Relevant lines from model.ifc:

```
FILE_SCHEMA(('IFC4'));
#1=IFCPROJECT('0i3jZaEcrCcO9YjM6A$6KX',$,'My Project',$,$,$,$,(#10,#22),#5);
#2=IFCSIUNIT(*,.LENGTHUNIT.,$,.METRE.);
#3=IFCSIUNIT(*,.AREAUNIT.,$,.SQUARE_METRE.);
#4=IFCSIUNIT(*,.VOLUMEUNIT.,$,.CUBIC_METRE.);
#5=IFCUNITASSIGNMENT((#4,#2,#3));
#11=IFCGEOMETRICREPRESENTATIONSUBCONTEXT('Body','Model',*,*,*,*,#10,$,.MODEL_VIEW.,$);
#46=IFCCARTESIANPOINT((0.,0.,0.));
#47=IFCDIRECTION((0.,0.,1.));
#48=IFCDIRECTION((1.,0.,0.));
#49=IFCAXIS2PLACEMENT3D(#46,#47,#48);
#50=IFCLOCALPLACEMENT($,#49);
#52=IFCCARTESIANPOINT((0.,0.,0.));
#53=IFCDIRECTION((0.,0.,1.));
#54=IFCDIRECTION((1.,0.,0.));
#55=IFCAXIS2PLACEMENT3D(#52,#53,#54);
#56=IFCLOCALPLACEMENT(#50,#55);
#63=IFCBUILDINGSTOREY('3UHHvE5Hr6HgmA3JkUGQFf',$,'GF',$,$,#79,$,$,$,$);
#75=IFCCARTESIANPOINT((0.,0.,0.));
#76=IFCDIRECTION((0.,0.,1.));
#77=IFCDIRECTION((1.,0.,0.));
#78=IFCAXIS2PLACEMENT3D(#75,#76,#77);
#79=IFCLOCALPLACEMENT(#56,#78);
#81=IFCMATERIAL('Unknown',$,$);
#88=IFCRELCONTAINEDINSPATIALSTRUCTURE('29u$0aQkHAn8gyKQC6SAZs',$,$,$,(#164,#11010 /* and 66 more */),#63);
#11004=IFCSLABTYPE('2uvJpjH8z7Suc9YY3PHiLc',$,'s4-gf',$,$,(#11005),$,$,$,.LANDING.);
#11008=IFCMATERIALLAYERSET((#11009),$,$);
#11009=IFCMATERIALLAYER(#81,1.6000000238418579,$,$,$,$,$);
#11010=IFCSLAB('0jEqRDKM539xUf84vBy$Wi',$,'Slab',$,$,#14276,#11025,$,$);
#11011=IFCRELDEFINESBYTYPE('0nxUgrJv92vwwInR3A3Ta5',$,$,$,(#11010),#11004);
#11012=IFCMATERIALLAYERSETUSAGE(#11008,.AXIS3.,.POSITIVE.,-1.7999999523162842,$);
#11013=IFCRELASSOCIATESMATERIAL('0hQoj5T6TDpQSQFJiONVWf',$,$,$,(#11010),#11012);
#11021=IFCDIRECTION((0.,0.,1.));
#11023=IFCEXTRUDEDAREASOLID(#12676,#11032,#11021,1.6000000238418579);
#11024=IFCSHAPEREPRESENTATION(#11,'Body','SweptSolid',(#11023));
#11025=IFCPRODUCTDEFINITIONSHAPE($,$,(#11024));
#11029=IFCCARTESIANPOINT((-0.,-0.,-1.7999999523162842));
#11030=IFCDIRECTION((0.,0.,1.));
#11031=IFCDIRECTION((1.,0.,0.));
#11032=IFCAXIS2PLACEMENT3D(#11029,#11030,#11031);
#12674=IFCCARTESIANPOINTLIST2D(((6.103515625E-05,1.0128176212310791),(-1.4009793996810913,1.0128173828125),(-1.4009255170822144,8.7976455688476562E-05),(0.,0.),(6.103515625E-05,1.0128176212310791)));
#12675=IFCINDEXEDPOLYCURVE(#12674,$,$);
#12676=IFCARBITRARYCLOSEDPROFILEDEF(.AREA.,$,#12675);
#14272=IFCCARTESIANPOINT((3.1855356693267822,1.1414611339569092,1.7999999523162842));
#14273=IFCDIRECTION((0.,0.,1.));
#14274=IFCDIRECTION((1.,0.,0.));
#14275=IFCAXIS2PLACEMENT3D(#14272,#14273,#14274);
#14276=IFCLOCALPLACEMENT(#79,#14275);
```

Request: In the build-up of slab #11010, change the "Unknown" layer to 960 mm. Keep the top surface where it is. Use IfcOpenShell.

```python
import ifcopenshell
import ifcopenshell.util.element
import ifcopenshell.util.representation
import ifcopenshell.util.unit

model = ifcopenshell.open("model.ifc")
unit_scale = ifcopenshell.util.unit.calculate_unit_scale(model)

layer_set = model.by_id(11008)
layer = next(l for l in layer_set.MaterialLayers if l.Material and l.Material.Name == "Unknown")
change = 0.96 / unit_scale - layer.LayerThickness
layer.LayerThickness += change

# Geometry does not follow the layer set by itself.
slabs = [e for e in ifcopenshell.util.element.get_elements_by_material(model, layer_set) if e.is_a("IfcSlab")]
for slab in sorted(slabs, key=lambda e: e.id()):
    body = ifcopenshell.util.representation.get_representation(slab, "Model", "Body")
    solid = body.Items[0]
    old_depth = solid.Depth
    solid.Depth += change
    # Extruded upwards: lower the start of the extrusion so the top stays.
    x, y, z = solid.Position.Location.Coordinates
    solid.Position.Location = model.createIfcCartesianPoint((x, y, z - change))
    print(slab.id(), f"{old_depth:g} -> {solid.Depth:g}")

# The layers are counted up from the underside, which has moved.
for usage in {ifcopenshell.util.element.get_material(slab) for slab in slabs}:
    usage.OffsetFromReferenceLine -= change

model.write("model_updated.ifc")
```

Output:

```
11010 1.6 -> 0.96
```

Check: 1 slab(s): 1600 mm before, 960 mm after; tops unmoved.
